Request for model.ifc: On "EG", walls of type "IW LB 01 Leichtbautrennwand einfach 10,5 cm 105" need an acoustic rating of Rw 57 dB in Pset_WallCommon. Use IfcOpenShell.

First a look at what the model holds.

```python
import ifcopenshell
import ifcopenshell.util.element

model = ifcopenshell.open("model.ifc")
print(model.schema)
storey = next(s for s in model.by_type("IfcBuildingStorey") if s.Name == "EG")
walls = [e for e in ifcopenshell.util.element.get_decomposition(storey) if e.is_a("IfcWall")]
seen = {}
for e in walls:
    element_type = ifcopenshell.util.element.get_type(e)
    key = (element_type.Name if element_type != e and element_type else None, ifcopenshell.util.element.get_pset(e, "Pset_WallCommon", "AcousticRating"))
    seen[key] = seen.get(key, 0) + 1
for (name, value), count in sorted(seen.items(), key=str):
    print(count, "x", name, "|", value)
```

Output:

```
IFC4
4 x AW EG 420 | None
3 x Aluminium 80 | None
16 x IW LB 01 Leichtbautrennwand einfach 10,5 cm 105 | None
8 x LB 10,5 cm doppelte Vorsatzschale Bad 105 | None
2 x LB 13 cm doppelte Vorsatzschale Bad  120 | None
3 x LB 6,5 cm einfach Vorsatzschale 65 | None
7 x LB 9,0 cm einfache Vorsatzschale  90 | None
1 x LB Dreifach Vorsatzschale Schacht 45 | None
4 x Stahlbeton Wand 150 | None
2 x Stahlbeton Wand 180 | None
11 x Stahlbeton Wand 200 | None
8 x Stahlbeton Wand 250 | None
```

```python
import ifcopenshell
import ifcopenshell.api.pset
import ifcopenshell.util.element

model = ifcopenshell.open("model.ifc")

storey = next(s for s in model.by_type("IfcBuildingStorey") if s.Name == "EG")
walls = [e for e in ifcopenshell.util.element.get_decomposition(storey) if e.is_a("IfcWall")]

count = 0
for e in walls:
    element_type = ifcopenshell.util.element.get_type(e)
    if element_type in (None, e) or element_type.Name != "IW LB 01 Leichtbautrennwand einfach 10,5 cm 105":
        continue
    # add_pset returns the element's existing set when there is one.
    pset = ifcopenshell.api.pset.add_pset(model, product=e, name="Pset_WallCommon")
    ifcopenshell.api.pset.edit_pset(model, pset=pset, properties={"AcousticRating": "Rw 57 dB"})
    count += 1

print(count, "walls updated")

model.write("model-out.ifc")
```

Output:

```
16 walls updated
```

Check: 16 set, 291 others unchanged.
